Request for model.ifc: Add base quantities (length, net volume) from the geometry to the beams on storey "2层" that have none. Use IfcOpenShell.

First a look at what the model holds.

```python
import ifcopenshell
import ifcopenshell.util.element
import ifcopenshell.util.unit

model = ifcopenshell.open("model.ifc")
print(model.schema)
for unit_type in ("LENGTHUNIT", "AREAUNIT", "VOLUMEUNIT"):
    print(unit_type, ifcopenshell.util.unit.calculate_unit_scale(model, unit_type))
storey = next(s for s in model.by_type("IfcBuildingStorey") if s.Name == "2层")
beams = [e for e in ifcopenshell.util.element.get_decomposition(storey) if e.is_a("IfcBeam")]
for e in sorted(beams, key=lambda e: e.id()):
    print(e.id(), e.is_a(), e.Name, list(ifcopenshell.util.element.get_psets(e, qtos_only=True)), sep=" | ")
```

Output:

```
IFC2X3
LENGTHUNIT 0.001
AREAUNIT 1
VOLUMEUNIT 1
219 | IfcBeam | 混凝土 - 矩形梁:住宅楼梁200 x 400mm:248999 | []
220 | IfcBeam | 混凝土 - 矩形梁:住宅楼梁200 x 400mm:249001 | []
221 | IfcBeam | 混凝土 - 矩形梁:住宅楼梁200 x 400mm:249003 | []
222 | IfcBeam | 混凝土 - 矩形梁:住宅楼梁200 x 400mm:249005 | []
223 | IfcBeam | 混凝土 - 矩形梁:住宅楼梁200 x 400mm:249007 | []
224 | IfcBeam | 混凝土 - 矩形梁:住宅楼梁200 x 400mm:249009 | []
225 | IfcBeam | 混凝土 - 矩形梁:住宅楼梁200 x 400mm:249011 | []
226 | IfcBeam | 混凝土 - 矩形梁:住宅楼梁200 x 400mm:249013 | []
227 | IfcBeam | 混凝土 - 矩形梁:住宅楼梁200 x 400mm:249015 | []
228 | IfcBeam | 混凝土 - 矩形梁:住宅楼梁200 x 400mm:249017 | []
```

```python
import ifcopenshell
import ifcopenshell.api.pset
import ifcopenshell.geom
import ifcopenshell.util.element
import ifcopenshell.util.shape
import ifcopenshell.util.unit

model = ifcopenshell.open("model.ifc")
unit_scale = ifcopenshell.util.unit.calculate_unit_scale(model)
volume_scale = ifcopenshell.util.unit.calculate_unit_scale(model, "VOLUMEUNIT")
settings = ifcopenshell.geom.settings()

storey = next(s for s in model.by_type("IfcBuildingStorey") if s.Name == "2层")
beams = [e for e in ifcopenshell.util.element.get_decomposition(storey) if e.is_a("IfcBeam")]

for e in sorted(beams, key=lambda e: e.id()):
    if ifcopenshell.util.element.get_psets(e, qtos_only=True, should_inherit=False):
        continue
    # Geometry comes back in metres, in the element's own axes.
    shape = ifcopenshell.geom.create_shape(settings, e)
    values = {
        "Length": ifcopenshell.util.shape.get_max_xyz(shape.geometry) / unit_scale,
        "NetVolume": ifcopenshell.util.shape.get_volume(shape.geometry) / volume_scale,
    }
    qto = ifcopenshell.api.pset.add_qto(model, product=e, name="BaseQuantities")
    ifcopenshell.api.pset.edit_qto(model, qto=qto, properties=values)
    print(e.id(), {k: round(v, 3) for k, v in values.items()})

model.write("model_edited.ifc")
```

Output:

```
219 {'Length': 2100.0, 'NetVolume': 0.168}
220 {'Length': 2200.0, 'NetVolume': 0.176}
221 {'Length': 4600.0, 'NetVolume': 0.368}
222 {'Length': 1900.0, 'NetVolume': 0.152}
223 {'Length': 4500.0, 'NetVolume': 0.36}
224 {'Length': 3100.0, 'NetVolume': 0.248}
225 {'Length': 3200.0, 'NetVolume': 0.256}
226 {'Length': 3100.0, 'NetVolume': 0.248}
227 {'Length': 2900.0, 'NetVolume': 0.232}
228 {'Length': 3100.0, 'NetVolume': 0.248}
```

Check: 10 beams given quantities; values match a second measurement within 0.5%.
